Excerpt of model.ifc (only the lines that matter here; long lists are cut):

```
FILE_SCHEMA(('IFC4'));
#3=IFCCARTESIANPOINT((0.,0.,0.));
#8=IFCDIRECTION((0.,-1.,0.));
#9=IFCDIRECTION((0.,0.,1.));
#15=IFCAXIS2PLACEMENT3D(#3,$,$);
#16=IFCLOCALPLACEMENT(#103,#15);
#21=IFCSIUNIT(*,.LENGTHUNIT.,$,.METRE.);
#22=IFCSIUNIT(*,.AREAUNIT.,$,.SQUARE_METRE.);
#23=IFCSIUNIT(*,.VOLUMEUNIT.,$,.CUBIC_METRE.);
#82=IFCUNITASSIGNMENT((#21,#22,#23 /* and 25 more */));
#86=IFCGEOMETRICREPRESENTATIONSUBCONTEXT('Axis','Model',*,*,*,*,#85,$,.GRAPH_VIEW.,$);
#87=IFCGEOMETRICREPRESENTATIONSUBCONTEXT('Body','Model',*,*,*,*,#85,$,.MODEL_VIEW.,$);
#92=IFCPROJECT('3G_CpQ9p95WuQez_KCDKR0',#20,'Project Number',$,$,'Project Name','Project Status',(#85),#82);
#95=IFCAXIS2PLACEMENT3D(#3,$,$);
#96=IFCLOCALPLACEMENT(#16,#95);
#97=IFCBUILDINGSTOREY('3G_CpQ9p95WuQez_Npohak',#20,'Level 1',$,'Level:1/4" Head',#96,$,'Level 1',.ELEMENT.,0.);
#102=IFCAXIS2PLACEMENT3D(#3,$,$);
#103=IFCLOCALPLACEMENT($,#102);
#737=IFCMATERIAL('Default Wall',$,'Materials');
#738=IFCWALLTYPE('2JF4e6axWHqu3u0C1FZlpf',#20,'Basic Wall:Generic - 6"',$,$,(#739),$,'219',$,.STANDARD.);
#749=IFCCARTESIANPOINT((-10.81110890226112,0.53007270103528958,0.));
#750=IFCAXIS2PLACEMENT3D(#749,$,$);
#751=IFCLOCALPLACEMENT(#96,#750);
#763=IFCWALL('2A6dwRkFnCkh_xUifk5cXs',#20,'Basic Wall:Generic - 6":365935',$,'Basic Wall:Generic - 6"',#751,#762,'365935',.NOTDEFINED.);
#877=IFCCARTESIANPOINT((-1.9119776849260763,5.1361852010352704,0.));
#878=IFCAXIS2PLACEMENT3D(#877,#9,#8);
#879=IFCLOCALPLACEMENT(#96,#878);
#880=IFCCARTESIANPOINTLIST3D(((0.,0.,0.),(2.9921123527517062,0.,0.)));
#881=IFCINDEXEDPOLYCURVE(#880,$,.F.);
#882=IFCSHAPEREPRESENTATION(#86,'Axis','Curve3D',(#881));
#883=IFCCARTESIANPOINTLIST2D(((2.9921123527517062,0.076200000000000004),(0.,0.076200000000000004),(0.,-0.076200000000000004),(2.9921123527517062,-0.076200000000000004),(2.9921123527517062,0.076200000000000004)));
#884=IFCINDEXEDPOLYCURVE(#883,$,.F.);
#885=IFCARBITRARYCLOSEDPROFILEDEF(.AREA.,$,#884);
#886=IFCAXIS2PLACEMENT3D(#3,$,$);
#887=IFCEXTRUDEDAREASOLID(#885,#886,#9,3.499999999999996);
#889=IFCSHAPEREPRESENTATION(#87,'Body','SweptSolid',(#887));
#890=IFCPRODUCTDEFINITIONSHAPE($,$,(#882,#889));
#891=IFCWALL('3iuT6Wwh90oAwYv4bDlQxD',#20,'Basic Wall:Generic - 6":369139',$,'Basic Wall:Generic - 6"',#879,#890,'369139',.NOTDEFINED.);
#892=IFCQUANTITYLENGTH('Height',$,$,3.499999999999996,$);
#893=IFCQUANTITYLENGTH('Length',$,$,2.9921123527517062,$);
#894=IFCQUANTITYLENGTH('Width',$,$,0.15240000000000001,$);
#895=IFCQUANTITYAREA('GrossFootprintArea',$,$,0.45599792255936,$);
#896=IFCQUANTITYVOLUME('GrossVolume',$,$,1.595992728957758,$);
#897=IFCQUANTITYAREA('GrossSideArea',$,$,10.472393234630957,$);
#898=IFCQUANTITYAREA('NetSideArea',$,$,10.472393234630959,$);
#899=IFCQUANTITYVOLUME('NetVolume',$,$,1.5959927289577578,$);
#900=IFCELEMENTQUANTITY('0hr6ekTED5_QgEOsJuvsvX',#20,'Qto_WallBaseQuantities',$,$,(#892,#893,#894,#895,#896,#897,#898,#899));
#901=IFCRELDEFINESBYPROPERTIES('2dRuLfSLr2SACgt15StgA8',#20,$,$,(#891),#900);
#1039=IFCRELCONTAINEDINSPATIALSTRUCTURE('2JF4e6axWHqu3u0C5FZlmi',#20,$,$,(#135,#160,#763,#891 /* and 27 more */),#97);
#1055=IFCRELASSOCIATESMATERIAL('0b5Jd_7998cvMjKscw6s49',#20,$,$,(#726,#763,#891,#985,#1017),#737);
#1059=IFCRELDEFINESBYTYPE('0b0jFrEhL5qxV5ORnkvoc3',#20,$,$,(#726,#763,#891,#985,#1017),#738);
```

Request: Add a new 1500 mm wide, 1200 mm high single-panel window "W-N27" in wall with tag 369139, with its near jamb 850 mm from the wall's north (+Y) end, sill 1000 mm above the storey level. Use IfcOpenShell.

```python
import numpy as np
import ifcopenshell
import ifcopenshell.api.feature
import ifcopenshell.api.geometry
import ifcopenshell.api.pset
import ifcopenshell.api.root
import ifcopenshell.api.spatial
import ifcopenshell.geom
import ifcopenshell.util.element
import ifcopenshell.util.placement
import ifcopenshell.util.representation
import ifcopenshell.util.shape
import ifcopenshell.util.unit

model = ifcopenshell.open("model.ifc")
unit_scale = ifcopenshell.util.unit.calculate_unit_scale(model)
area_scale = ifcopenshell.util.unit.calculate_unit_scale(model, "AREAUNIT")
volume_scale = ifcopenshell.util.unit.calculate_unit_scale(model, "VOLUMEUNIT")
settings = ifcopenshell.geom.settings()


def volume(element):
    """Net volume in cubic metres, openings subtracted."""
    shape = ifcopenshell.geom.create_shape(settings, element)
    return ifcopenshell.util.shape.get_volume(shape.geometry)


wall = model.by_id(891)
storey = ifcopenshell.util.element.get_container(wall, ifc_class="IfcBuildingStorey")
context = ifcopenshell.util.representation.get_context(model, "Model", "Body", "MODEL_VIEW")
before = volume(wall)

width, height, from_end, sill = 1.5, 1.2, 0.85, 1  # metres

# The wall runs along its own X axis, and the end named is its -X end.
wall_shape = ifcopenshell.geom.create_shape(settings, wall)
x, y, z = ifcopenshell.util.shape.get_vertices(wall_shape.geometry).T
start = x.min() + from_end
face, thickness = float(y.min()), float(y.max() - y.min())
wall_matrix = ifcopenshell.util.placement.get_local_placement(wall.ObjectPlacement)
level = ifcopenshell.util.placement.get_local_placement(storey.ObjectPlacement)[2, 3]


def in_wall(x, y):
    """Placement at x, y metres in the wall's axes, at sill height."""
    matrix = wall_matrix.copy()
    matrix[:, 3] = wall_matrix @ np.array([x / unit_scale, y / unit_scale, 0.0, 1.0])
    matrix[2, 3] = level + sill / unit_scale
    return matrix


# Opening: a box that overshoots both wall faces by 50 mm.
opening = ifcopenshell.api.root.create_entity(model, ifc_class="IfcOpeningElement", predefined_type="OPENING")
box = ifcopenshell.api.geometry.add_wall_representation(
    model, context=context, length=width, height=height, thickness=thickness + 0.1
)
ifcopenshell.api.geometry.assign_representation(model, product=opening, representation=box)
ifcopenshell.api.geometry.edit_object_placement(model, product=opening, matrix=in_wall(start, face - 0.05), is_si=False)
ifcopenshell.api.feature.add_feature(model, feature=opening, element=wall)

window = ifcopenshell.api.root.create_entity(model, ifc_class="IfcWindow", name="W-N27", predefined_type="WINDOW")
window.OverallWidth, window.OverallHeight = width / unit_scale, height / unit_scale
window.PartitioningType = "SINGLE_PANEL"
body = ifcopenshell.api.geometry.add_window_representation(
    model,
    context=context,
    overall_width=window.OverallWidth,
    overall_height=window.OverallHeight,
    partition_type="SINGLE_PANEL",
)
ifcopenshell.api.geometry.assign_representation(model, product=window, representation=body)
ifcopenshell.api.spatial.assign_container(model, products=[window], relating_structure=storey)
ifcopenshell.api.feature.add_filling(model, opening=opening, element=window)

# Centre the window in the wall's thickness.
ifcopenshell.api.geometry.edit_object_placement(model, product=window, matrix=in_wall(start, face), is_si=False)
window_shape = ifcopenshell.geom.create_shape(settings, window)
depth = ifcopenshell.util.shape.get_vertices(window_shape.geometry)[:, 1]
offset = face + thickness / 2 - (depth.min() + depth.max()) / 2
ifcopenshell.api.geometry.edit_object_placement(model, product=window, matrix=in_wall(start, offset), is_si=False)

after = volume(wall)

# Update the wall's stored quantities.
qto = model.by_id(ifcopenshell.util.element.get_pset(wall, "Qto_WallBaseQuantities", should_inherit=False)["id"])
ifcopenshell.api.pset.edit_qto(model, qto=qto, properties={
    "NetSideArea": after / thickness / area_scale,
    "NetVolume": after / volume_scale,
})

print(f"wall volume {before:.3f} -> {after:.3f} m3")

model.write("model_v2.ifc")
```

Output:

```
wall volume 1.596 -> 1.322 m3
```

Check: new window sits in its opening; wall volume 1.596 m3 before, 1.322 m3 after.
